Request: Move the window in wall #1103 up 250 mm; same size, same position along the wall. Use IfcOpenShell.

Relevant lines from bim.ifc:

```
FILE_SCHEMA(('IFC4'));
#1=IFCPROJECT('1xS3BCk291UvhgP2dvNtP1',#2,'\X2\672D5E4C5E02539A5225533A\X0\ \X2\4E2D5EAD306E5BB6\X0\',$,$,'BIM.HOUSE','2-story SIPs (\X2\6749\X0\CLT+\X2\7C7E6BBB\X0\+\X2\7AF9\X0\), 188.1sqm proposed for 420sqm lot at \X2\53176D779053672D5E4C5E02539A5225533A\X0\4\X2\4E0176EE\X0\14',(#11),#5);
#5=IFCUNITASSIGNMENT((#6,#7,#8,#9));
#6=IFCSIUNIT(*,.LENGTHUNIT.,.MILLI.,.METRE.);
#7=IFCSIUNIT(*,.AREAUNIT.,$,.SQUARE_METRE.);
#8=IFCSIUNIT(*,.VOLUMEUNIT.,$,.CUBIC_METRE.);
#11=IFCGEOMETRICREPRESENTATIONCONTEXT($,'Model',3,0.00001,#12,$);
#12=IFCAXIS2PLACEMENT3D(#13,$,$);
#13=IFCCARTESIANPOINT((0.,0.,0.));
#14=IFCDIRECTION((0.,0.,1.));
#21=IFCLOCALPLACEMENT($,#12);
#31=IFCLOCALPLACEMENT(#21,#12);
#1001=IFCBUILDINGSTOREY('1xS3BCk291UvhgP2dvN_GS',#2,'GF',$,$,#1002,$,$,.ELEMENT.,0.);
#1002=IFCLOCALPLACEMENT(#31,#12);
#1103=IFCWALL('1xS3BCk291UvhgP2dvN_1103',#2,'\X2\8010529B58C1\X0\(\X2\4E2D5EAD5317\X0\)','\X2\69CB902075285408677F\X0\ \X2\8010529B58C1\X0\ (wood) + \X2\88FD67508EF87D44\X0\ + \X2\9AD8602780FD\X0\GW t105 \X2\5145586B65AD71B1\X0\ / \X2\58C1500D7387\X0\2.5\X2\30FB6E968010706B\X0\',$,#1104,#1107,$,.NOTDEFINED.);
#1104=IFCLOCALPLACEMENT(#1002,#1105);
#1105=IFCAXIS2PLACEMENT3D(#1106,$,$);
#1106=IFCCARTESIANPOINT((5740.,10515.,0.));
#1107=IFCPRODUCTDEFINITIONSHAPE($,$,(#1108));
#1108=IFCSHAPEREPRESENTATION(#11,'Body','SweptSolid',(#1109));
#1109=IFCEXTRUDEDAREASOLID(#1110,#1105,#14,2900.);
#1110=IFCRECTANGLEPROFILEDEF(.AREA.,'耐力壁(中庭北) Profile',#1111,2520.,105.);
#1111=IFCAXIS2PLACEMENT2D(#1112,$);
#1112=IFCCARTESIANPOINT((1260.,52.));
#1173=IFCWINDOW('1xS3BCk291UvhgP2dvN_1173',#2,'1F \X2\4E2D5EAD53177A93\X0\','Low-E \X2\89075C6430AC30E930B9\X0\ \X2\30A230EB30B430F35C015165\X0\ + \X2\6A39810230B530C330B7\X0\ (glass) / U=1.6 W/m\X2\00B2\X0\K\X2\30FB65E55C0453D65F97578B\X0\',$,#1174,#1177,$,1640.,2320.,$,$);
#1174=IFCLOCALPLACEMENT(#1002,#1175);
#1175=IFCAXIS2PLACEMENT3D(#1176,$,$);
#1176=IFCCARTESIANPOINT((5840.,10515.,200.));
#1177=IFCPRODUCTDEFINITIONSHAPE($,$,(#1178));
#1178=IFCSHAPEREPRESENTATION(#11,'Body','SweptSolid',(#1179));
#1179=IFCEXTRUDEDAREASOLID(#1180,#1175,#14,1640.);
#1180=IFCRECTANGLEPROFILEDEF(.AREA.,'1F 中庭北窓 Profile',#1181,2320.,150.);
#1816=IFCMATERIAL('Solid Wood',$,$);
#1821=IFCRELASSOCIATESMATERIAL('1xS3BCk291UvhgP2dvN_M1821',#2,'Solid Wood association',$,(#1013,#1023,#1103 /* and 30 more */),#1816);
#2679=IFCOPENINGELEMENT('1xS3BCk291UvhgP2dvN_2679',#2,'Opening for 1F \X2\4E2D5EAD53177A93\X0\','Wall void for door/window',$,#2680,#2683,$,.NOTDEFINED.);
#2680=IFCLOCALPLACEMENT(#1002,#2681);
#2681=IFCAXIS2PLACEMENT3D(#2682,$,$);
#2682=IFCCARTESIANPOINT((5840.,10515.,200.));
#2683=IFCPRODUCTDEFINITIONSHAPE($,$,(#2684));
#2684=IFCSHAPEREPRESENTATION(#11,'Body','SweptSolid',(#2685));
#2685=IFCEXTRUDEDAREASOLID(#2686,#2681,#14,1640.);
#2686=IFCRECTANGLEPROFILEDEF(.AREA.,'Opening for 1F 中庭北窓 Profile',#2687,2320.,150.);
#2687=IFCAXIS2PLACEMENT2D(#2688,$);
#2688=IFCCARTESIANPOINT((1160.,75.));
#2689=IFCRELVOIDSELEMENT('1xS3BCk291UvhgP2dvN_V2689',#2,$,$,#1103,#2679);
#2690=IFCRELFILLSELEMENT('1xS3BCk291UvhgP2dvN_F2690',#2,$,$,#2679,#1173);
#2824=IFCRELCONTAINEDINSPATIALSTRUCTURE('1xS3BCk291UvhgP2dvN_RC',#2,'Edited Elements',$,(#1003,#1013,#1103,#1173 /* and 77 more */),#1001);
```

```python
import numpy as np
import ifcopenshell
import ifcopenshell.api.geometry
import ifcopenshell.util.placement
import ifcopenshell.util.unit

model = ifcopenshell.open("bim.ifc")
unit_scale = ifcopenshell.util.unit.calculate_unit_scale(model)

window = model.by_guid("1xS3BCk291UvhgP2dvN_1173")
opening = window.FillsVoids[0].RelatingOpeningElement
dz = 0.25 / unit_scale

shift = np.array([0.0, 0.0, dz])
# The window is not placed relative to its opening, so move both.
for product in (opening, window):
    matrix = ifcopenshell.util.placement.get_local_placement(product.ObjectPlacement)
    matrix[:3, 3] += shift
    ifcopenshell.api.geometry.edit_object_placement(model, product=product, matrix=matrix, is_si=False)

print(f"moved by {dz * unit_scale:+.3f} m")

model.write("bim_updated.ifc")
```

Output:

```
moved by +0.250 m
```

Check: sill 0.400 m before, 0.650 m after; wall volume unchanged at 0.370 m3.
